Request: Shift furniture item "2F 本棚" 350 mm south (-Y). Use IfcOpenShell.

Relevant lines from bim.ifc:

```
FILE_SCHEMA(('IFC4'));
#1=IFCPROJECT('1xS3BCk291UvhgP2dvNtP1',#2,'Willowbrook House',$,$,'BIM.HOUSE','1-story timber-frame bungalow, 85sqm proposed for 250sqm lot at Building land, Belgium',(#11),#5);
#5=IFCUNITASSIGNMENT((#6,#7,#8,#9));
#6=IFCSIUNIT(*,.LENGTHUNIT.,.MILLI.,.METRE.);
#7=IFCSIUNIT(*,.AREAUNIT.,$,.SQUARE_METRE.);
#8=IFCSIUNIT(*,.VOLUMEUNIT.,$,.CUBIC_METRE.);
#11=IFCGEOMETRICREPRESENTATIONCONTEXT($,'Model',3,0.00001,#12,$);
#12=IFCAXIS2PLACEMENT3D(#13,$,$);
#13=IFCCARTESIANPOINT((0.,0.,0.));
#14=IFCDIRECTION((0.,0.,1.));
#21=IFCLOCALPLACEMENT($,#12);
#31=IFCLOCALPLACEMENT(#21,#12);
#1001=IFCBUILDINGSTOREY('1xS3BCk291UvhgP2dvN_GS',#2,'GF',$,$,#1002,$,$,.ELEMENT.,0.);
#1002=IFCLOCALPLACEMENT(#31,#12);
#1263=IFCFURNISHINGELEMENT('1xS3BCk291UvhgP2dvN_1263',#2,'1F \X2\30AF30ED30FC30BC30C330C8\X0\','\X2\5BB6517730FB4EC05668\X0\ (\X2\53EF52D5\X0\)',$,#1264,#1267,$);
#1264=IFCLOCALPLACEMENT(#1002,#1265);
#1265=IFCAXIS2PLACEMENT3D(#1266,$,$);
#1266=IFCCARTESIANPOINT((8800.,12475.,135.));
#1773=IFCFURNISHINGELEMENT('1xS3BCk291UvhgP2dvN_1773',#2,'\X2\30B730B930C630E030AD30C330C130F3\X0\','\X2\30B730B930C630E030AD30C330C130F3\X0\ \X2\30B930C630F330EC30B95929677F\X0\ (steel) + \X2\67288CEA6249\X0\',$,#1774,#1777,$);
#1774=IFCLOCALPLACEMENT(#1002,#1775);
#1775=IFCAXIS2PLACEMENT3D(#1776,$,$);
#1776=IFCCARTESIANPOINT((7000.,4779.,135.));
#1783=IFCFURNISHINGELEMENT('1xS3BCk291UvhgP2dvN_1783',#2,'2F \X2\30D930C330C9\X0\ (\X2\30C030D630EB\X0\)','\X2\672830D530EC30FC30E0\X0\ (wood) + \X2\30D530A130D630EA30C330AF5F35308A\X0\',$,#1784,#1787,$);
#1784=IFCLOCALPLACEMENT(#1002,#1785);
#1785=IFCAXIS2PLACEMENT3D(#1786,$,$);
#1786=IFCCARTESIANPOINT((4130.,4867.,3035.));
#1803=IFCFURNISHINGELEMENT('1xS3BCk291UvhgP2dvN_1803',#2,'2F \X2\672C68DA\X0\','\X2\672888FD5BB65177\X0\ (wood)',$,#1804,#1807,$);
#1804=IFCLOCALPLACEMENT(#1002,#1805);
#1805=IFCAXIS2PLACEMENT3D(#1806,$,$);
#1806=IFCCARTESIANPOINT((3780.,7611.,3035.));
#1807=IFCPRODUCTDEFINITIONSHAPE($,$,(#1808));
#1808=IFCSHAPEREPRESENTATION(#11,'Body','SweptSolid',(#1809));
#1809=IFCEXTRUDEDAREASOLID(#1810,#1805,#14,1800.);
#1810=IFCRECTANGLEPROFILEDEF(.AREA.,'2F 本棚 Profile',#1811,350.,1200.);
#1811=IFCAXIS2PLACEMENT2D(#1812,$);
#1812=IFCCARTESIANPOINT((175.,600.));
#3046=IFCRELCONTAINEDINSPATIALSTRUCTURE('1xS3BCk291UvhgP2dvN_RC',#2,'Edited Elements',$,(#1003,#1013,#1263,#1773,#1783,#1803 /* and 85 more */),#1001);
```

```python
import ifcopenshell
import ifcopenshell.api.geometry
import ifcopenshell.util.placement
import ifcopenshell.util.unit

model = ifcopenshell.open("bim.ifc")
unit_scale = ifcopenshell.util.unit.calculate_unit_scale(model)

item = model.by_guid("1xS3BCk291UvhgP2dvN_1803")
matrix = ifcopenshell.util.placement.get_local_placement(item.ObjectPlacement)
matrix[1, 3] -= 0.35 / unit_scale
ifcopenshell.api.geometry.edit_object_placement(model, product=item, matrix=matrix, is_si=False)

print(ifcopenshell.util.placement.get_local_placement(item.ObjectPlacement).round(3) + 0.0)

model.write("bim_updated.ifc")
```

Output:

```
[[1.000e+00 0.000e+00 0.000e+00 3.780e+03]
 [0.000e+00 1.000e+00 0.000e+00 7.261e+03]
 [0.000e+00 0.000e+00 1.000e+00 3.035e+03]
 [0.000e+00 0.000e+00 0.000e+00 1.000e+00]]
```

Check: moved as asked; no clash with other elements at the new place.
